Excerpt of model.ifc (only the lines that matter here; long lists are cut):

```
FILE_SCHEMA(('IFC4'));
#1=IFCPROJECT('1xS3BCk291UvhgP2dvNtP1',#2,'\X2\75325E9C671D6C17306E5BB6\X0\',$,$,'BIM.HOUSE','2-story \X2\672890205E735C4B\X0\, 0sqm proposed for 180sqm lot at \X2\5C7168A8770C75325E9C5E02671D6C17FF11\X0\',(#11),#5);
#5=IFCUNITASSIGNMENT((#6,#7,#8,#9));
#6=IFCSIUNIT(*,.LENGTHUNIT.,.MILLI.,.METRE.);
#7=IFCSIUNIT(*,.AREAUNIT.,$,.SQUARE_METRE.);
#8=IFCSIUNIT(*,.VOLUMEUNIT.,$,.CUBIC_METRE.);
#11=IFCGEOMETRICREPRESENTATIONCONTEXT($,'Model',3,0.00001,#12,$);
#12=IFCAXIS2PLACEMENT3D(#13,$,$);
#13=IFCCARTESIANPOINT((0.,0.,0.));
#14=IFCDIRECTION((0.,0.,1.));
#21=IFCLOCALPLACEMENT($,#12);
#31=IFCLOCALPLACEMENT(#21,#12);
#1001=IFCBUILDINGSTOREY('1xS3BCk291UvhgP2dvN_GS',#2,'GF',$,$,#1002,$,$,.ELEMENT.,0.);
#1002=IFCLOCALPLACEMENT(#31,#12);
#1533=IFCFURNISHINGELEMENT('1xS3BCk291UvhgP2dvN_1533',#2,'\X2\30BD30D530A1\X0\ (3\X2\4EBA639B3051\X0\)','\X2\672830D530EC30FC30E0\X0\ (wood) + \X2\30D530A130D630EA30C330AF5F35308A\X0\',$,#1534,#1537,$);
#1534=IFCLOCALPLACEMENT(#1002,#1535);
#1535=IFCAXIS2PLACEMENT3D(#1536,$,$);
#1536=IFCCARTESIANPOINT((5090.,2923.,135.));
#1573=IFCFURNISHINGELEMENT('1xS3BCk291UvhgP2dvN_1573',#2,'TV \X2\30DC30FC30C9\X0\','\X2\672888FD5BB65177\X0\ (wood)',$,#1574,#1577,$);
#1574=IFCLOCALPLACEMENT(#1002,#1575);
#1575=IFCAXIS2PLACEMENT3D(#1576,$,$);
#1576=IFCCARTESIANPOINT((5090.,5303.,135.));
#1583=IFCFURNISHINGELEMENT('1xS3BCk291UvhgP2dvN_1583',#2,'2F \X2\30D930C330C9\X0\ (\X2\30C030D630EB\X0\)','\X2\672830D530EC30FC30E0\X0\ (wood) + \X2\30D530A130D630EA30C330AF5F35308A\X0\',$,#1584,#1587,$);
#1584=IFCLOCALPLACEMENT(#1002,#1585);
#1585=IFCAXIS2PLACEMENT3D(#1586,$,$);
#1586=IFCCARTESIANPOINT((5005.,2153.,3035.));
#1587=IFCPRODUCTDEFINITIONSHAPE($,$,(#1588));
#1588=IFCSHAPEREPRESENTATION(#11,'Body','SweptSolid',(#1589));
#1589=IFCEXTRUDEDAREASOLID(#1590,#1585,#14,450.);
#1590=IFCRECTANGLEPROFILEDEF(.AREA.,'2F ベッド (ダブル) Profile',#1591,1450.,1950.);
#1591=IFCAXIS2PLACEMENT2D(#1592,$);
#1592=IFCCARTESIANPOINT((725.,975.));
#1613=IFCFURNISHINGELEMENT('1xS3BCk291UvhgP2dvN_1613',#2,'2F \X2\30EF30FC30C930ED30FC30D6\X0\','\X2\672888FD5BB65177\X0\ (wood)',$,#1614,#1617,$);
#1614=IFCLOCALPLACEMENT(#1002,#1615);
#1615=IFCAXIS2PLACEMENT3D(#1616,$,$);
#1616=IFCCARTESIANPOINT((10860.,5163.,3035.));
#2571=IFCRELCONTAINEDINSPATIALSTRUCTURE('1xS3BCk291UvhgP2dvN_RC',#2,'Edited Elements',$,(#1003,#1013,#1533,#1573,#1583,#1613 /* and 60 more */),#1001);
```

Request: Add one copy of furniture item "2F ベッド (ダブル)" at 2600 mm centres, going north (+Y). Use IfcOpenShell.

```python
import numpy as np
import ifcopenshell
import ifcopenshell.api.geometry
import ifcopenshell.api.root
import ifcopenshell.util.element
import ifcopenshell.util.placement
import ifcopenshell.util.unit

model = ifcopenshell.open("model.ifc")
unit_scale = ifcopenshell.util.unit.calculate_unit_scale(model)


def reuse_history(source, copy):
    """copy_class also copies each property set's owner history, people and application; keep the originals."""
    for rel in copy.IsDefinedBy:
        if rel.is_a("IfcRelDefinesByProperties") and (history := rel.RelatingPropertyDefinition.OwnerHistory):
            rel.RelatingPropertyDefinition.OwnerHistory = source.OwnerHistory
            ifcopenshell.util.element.remove_deep2(model, history)


source = model.by_guid("1xS3BCk291UvhgP2dvN_1583")
base = ifcopenshell.util.placement.get_local_placement(source.ObjectPlacement)
step = np.array([0.0, 1.0, 0.0]) * 2.6 / unit_scale

for i in range(1, 2):
    copy = ifcopenshell.api.root.copy_class(model, product=source)
    copy.Representation = ifcopenshell.util.element.copy_deep(
        model, source.Representation, exclude=["IfcGeometricRepresentationContext", "IfcRepresentationMap"]
    )
    reuse_history(source, copy)
    matrix = base.copy()
    matrix[:3, 3] += i * step
    print("added at", matrix[:3, 3].round(3) + 0.0)
    ifcopenshell.api.geometry.edit_object_placement(model, product=copy, matrix=matrix, is_si=False)

model.write("model_rev.ifc")
```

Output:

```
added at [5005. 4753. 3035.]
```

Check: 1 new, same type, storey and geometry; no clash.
